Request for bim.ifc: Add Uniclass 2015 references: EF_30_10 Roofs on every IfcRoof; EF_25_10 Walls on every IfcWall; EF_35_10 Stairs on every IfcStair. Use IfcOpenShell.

First a look at what the model holds.

```python
import ifcopenshell

model = ifcopenshell.open("bim.ifc")
print(model.schema)
print("classifications:", [c.Name for c in model.by_type("IfcClassification")])
for ifc_class in ("IfcDoor", "IfcRoof", "IfcStair", "IfcWall", "IfcWindow"):
    print(ifc_class, len(model.by_type(ifc_class)))
```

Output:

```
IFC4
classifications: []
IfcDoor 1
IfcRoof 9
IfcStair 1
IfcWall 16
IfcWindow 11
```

```python
import ifcopenshell
import ifcopenshell.api.classification

model = ifcopenshell.open("bim.ifc")

system = ifcopenshell.api.classification.add_classification(model, classification="Uniclass 2015")

codes = {
    "IfcRoof": ("EF_30_10", "Roofs"),
    "IfcWall": ("EF_25_10", "Walls"),
    "IfcStair": ("EF_35_10", "Stairs"),
}
for ifc_class, (code, name) in codes.items():
    products = model.by_type(ifc_class)
    ifcopenshell.api.classification.add_reference(
        model, products=products, classification=system, identification=code, name=name
    )
    print(code, len(products))

model.write("bim_rev.ifc")
```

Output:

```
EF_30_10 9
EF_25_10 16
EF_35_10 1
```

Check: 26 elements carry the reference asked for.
